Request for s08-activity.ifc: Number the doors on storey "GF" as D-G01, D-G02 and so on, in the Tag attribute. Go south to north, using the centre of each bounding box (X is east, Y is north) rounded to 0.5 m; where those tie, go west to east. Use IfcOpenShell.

First a look at what the model holds.

```python
import ifcopenshell
import ifcopenshell.util.element
import ifcopenshell.util.placement

model = ifcopenshell.open("s08-activity.ifc")
print(model.schema)
storey = next(s for s in model.by_type("IfcBuildingStorey") if s.Name == "GF")
doors = [e for e in ifcopenshell.util.element.get_decomposition(storey) if e.is_a("IfcDoor")]
for e in sorted(doors, key=lambda e: e.id()):
    origin = ifcopenshell.util.placement.get_local_placement(e.ObjectPlacement)[:3, 3]
    print(e.id(), e.Tag, e.Name, origin.round(2) + 0.0, sep=" | ")
```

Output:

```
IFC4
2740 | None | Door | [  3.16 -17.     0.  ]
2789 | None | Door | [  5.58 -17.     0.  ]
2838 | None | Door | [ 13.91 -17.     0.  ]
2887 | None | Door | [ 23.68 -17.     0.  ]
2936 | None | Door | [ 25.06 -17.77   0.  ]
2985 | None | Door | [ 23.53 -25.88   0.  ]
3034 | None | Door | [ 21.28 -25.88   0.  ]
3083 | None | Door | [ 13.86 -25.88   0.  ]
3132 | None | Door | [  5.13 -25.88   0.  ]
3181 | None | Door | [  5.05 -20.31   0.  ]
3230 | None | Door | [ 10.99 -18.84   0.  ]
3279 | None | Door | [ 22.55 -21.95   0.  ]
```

```python
import ifcopenshell
import ifcopenshell.geom
import ifcopenshell.util.element
import ifcopenshell.util.shape

model = ifcopenshell.open("s08-activity.ifc")
settings = ifcopenshell.geom.settings()
settings.set("use-world-coords", True)


def centre(element):
    shape = ifcopenshell.geom.create_shape(settings, element)
    return ifcopenshell.util.shape.get_bbox_centroid(shape.geometry)


storey = next(s for s in model.by_type("IfcBuildingStorey") if s.Name == "GF")
doors = [e for e in ifcopenshell.util.element.get_decomposition(storey) if e.is_a("IfcDoor")]

# Insertion points can sit at a corner or the storey origin, so sort by the geometry (in metres).
centres = {e: centre(e) for e in doors}
doors.sort(key=lambda e: (round(centres[e][1] / 0.5), centres[e][0]))

for i, e in enumerate(doors, start=1):
    number = f"D-G{i:02d}"
    e.Tag = number
    print(e.id(), number)

model.write("s08-activity_rev.ifc")
```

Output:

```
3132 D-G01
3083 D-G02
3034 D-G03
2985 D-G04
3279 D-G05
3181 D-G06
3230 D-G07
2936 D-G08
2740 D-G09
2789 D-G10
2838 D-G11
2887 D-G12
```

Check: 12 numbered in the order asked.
